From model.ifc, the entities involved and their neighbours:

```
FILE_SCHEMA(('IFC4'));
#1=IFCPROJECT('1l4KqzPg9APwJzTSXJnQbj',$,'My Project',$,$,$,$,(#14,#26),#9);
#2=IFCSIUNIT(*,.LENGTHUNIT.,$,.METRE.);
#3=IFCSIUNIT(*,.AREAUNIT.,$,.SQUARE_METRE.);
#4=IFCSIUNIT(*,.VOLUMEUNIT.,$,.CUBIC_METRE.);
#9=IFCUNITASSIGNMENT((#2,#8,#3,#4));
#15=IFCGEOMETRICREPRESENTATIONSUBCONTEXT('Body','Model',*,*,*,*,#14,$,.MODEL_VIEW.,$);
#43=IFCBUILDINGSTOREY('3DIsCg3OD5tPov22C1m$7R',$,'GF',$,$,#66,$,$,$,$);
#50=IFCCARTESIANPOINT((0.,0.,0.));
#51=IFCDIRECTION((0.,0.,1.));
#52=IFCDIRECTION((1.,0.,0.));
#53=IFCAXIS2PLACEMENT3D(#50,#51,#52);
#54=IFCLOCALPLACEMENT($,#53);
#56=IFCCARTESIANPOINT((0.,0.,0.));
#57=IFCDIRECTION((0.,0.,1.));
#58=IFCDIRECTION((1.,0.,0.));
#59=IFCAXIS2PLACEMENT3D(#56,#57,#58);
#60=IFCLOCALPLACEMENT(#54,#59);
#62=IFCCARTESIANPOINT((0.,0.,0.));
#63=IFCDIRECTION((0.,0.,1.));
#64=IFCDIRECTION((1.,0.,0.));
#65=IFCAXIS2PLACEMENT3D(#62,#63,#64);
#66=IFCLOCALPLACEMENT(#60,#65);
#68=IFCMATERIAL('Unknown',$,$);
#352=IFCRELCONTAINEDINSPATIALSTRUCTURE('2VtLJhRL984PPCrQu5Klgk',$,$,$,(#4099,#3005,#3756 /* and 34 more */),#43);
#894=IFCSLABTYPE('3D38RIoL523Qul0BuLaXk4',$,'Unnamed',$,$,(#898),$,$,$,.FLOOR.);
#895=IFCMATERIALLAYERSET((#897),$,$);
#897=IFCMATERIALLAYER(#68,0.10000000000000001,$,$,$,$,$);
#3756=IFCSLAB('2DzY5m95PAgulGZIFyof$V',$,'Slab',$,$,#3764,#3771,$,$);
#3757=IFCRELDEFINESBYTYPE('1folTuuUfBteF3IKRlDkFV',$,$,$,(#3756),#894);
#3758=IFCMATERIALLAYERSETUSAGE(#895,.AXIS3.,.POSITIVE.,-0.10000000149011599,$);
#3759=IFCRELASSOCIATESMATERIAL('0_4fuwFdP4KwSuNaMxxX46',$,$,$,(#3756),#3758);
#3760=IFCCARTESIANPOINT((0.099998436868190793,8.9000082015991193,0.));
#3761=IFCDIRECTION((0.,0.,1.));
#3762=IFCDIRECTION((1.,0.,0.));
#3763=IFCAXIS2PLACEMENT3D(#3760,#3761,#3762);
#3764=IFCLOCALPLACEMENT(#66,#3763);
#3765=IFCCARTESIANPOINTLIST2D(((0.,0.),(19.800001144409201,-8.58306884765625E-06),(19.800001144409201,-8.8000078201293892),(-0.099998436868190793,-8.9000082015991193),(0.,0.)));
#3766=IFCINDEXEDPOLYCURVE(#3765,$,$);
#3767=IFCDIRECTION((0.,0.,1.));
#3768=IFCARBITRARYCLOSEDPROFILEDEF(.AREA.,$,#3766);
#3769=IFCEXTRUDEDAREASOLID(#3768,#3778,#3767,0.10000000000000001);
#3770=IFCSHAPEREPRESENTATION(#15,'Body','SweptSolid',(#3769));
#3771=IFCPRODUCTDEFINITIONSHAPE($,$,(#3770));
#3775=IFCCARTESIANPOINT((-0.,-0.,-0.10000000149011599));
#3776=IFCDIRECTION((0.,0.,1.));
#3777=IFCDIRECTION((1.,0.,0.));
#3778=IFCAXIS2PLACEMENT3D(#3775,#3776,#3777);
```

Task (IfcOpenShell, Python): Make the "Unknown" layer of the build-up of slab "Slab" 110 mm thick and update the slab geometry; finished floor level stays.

```python
import ifcopenshell
import ifcopenshell.util.element
import ifcopenshell.util.representation
import ifcopenshell.util.unit

model = ifcopenshell.open("model.ifc")
unit_scale = ifcopenshell.util.unit.calculate_unit_scale(model)

layer_set = model.by_id(895)
layer = next(l for l in layer_set.MaterialLayers if l.Material and l.Material.Name == "Unknown")
change = 0.11 / unit_scale - layer.LayerThickness
layer.LayerThickness += change

# Geometry does not follow the layer set by itself.
slabs = [e for e in ifcopenshell.util.element.get_elements_by_material(model, layer_set) if e.is_a("IfcSlab")]
for slab in sorted(slabs, key=lambda e: e.id()):
    body = ifcopenshell.util.representation.get_representation(slab, "Model", "Body")
    solid = body.Items[0]
    old_depth = solid.Depth
    solid.Depth += change
    # Extruded upwards: lower the start of the extrusion so the top stays.
    x, y, z = solid.Position.Location.Coordinates
    solid.Position.Location = model.createIfcCartesianPoint((x, y, z - change))
    print(slab.id(), f"{old_depth:g} -> {solid.Depth:g}")

# The layers are counted up from the underside, which has moved.
for usage in {ifcopenshell.util.element.get_material(slab) for slab in slabs}:
    usage.OffsetFromReferenceLine -= change

model.write("model_v2.ifc")
```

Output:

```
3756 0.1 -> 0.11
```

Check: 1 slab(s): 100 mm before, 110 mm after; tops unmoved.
